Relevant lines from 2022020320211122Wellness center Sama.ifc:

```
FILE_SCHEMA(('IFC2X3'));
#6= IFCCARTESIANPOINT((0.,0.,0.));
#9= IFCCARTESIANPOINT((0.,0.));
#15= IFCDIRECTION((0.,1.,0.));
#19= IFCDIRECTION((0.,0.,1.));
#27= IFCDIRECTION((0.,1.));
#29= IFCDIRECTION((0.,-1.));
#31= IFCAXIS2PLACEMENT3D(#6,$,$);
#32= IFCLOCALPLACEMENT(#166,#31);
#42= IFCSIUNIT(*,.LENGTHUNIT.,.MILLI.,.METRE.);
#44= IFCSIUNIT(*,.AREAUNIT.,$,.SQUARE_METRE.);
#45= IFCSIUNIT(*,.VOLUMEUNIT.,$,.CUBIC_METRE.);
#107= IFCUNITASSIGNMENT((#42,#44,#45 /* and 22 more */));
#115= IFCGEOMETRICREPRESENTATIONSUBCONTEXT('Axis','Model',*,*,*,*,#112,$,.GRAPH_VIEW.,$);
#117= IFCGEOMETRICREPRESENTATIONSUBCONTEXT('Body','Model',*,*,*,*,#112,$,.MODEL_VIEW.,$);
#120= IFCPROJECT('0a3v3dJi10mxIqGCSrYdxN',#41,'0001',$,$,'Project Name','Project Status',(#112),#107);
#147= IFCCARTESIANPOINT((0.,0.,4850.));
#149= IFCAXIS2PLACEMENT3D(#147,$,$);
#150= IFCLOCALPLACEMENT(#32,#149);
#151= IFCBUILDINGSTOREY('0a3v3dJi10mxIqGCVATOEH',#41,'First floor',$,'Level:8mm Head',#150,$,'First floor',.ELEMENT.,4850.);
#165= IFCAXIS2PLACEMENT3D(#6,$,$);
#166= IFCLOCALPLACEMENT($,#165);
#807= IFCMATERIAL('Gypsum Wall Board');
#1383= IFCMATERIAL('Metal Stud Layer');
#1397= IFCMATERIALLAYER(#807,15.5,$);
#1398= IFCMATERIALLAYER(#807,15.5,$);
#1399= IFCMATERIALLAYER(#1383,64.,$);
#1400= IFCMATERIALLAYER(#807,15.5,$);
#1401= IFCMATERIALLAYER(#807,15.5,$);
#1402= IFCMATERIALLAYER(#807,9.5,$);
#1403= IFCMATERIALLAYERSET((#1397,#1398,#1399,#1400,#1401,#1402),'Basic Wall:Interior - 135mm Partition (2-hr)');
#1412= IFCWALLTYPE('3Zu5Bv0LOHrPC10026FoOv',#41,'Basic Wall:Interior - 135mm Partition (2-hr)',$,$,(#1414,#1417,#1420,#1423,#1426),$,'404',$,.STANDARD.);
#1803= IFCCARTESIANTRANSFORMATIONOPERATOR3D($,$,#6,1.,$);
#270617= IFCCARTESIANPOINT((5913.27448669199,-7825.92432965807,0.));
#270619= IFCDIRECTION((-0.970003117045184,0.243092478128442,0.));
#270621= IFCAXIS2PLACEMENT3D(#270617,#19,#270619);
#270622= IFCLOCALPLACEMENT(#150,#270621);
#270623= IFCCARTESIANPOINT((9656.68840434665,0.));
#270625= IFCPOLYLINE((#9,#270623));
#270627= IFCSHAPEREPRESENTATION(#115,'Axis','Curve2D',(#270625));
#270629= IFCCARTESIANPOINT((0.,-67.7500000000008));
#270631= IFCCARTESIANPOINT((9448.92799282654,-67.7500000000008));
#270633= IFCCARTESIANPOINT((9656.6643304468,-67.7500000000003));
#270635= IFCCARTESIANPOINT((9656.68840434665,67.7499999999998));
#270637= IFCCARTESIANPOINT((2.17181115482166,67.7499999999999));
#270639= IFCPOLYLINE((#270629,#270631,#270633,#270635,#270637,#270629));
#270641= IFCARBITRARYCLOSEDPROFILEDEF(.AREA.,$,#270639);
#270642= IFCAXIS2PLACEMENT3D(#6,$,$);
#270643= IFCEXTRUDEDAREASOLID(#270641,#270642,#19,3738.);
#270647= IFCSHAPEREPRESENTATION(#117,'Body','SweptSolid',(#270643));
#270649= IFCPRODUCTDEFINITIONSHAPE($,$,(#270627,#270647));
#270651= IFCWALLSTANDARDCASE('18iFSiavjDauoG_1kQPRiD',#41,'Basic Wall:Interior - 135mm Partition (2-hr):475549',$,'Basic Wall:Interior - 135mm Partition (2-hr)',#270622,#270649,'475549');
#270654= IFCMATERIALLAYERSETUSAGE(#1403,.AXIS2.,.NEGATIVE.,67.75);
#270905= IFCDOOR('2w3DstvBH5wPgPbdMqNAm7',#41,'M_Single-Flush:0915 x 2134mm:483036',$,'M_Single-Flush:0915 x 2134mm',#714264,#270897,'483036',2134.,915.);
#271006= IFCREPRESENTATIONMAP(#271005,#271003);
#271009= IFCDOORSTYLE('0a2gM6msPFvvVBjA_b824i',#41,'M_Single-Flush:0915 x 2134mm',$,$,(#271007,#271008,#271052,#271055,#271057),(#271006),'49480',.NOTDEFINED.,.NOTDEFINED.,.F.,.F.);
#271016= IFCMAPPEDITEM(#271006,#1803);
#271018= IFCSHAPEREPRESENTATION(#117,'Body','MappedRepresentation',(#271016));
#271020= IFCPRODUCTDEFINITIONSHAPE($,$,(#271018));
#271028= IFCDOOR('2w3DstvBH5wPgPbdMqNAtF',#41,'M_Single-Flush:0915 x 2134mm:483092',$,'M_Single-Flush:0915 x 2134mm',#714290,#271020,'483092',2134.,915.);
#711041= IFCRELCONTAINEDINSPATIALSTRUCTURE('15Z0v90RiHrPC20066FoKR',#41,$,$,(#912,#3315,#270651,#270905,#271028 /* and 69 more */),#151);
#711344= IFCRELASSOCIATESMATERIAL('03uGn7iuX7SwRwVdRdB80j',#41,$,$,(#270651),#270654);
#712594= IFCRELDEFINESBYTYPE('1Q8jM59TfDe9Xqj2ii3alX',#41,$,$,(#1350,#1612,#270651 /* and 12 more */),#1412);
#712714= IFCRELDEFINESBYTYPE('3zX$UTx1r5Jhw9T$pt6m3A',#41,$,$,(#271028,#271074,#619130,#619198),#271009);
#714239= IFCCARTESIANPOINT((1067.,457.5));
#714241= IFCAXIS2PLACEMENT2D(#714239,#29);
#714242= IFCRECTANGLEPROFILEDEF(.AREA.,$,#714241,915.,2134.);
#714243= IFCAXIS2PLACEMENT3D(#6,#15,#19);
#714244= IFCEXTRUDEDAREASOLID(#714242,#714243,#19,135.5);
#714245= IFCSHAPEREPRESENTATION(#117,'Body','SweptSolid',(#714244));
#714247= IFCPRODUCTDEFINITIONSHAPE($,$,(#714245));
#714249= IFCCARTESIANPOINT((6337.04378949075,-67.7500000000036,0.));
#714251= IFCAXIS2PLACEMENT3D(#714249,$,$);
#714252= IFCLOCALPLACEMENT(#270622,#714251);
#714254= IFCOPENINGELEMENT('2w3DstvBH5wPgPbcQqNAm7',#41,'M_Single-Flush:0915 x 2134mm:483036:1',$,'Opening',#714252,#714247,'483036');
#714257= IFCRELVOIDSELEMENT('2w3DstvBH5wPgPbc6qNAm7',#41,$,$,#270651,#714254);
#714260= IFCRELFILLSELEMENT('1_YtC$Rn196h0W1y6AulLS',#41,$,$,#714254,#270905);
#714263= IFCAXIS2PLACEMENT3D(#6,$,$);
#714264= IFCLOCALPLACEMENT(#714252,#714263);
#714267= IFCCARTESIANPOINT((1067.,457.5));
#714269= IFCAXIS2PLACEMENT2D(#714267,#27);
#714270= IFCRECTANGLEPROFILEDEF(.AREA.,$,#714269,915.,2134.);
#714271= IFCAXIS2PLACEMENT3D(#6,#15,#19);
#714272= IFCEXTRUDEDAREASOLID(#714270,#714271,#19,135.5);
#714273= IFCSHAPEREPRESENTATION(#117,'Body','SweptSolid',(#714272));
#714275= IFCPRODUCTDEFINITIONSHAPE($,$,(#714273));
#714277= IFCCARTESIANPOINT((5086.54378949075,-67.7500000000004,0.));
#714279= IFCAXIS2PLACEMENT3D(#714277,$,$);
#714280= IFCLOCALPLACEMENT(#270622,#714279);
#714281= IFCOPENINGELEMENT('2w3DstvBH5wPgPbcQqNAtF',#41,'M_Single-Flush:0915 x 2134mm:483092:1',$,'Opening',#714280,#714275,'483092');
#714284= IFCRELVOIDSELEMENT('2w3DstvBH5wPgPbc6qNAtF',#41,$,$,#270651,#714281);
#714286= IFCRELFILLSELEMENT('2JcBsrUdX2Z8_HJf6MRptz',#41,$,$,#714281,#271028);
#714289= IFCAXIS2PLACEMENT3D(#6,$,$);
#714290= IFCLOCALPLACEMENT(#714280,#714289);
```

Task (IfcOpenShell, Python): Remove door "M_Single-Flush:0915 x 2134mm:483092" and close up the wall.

```python
import ifcopenshell
import ifcopenshell.api.feature
import ifcopenshell.api.root
import ifcopenshell.geom
import ifcopenshell.util.shape

model = ifcopenshell.open("2022020320211122Wellness center Sama.ifc")
settings = ifcopenshell.geom.settings()


def volume(element):
    """Net volume in cubic metres, openings subtracted."""
    shape = ifcopenshell.geom.create_shape(settings, element)
    return ifcopenshell.util.shape.get_volume(shape.geometry)


door = model.by_guid("2w3DstvBH5wPgPbdMqNAtF")
opening = door.FillsVoids[0].RelatingOpeningElement
wall = opening.VoidsElements[0].RelatingBuildingElement
before = volume(wall)

ifcopenshell.api.root.remove_product(model, product=door)
ifcopenshell.api.feature.remove_feature(model, feature=opening)

after = volume(wall)

print(f"wall volume {before:.3f} -> {after:.3f} m3")

model.write("2022020320211122Wellness center Sama_v2.ifc")
```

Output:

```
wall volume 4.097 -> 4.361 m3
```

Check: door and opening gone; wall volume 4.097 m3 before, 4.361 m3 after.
